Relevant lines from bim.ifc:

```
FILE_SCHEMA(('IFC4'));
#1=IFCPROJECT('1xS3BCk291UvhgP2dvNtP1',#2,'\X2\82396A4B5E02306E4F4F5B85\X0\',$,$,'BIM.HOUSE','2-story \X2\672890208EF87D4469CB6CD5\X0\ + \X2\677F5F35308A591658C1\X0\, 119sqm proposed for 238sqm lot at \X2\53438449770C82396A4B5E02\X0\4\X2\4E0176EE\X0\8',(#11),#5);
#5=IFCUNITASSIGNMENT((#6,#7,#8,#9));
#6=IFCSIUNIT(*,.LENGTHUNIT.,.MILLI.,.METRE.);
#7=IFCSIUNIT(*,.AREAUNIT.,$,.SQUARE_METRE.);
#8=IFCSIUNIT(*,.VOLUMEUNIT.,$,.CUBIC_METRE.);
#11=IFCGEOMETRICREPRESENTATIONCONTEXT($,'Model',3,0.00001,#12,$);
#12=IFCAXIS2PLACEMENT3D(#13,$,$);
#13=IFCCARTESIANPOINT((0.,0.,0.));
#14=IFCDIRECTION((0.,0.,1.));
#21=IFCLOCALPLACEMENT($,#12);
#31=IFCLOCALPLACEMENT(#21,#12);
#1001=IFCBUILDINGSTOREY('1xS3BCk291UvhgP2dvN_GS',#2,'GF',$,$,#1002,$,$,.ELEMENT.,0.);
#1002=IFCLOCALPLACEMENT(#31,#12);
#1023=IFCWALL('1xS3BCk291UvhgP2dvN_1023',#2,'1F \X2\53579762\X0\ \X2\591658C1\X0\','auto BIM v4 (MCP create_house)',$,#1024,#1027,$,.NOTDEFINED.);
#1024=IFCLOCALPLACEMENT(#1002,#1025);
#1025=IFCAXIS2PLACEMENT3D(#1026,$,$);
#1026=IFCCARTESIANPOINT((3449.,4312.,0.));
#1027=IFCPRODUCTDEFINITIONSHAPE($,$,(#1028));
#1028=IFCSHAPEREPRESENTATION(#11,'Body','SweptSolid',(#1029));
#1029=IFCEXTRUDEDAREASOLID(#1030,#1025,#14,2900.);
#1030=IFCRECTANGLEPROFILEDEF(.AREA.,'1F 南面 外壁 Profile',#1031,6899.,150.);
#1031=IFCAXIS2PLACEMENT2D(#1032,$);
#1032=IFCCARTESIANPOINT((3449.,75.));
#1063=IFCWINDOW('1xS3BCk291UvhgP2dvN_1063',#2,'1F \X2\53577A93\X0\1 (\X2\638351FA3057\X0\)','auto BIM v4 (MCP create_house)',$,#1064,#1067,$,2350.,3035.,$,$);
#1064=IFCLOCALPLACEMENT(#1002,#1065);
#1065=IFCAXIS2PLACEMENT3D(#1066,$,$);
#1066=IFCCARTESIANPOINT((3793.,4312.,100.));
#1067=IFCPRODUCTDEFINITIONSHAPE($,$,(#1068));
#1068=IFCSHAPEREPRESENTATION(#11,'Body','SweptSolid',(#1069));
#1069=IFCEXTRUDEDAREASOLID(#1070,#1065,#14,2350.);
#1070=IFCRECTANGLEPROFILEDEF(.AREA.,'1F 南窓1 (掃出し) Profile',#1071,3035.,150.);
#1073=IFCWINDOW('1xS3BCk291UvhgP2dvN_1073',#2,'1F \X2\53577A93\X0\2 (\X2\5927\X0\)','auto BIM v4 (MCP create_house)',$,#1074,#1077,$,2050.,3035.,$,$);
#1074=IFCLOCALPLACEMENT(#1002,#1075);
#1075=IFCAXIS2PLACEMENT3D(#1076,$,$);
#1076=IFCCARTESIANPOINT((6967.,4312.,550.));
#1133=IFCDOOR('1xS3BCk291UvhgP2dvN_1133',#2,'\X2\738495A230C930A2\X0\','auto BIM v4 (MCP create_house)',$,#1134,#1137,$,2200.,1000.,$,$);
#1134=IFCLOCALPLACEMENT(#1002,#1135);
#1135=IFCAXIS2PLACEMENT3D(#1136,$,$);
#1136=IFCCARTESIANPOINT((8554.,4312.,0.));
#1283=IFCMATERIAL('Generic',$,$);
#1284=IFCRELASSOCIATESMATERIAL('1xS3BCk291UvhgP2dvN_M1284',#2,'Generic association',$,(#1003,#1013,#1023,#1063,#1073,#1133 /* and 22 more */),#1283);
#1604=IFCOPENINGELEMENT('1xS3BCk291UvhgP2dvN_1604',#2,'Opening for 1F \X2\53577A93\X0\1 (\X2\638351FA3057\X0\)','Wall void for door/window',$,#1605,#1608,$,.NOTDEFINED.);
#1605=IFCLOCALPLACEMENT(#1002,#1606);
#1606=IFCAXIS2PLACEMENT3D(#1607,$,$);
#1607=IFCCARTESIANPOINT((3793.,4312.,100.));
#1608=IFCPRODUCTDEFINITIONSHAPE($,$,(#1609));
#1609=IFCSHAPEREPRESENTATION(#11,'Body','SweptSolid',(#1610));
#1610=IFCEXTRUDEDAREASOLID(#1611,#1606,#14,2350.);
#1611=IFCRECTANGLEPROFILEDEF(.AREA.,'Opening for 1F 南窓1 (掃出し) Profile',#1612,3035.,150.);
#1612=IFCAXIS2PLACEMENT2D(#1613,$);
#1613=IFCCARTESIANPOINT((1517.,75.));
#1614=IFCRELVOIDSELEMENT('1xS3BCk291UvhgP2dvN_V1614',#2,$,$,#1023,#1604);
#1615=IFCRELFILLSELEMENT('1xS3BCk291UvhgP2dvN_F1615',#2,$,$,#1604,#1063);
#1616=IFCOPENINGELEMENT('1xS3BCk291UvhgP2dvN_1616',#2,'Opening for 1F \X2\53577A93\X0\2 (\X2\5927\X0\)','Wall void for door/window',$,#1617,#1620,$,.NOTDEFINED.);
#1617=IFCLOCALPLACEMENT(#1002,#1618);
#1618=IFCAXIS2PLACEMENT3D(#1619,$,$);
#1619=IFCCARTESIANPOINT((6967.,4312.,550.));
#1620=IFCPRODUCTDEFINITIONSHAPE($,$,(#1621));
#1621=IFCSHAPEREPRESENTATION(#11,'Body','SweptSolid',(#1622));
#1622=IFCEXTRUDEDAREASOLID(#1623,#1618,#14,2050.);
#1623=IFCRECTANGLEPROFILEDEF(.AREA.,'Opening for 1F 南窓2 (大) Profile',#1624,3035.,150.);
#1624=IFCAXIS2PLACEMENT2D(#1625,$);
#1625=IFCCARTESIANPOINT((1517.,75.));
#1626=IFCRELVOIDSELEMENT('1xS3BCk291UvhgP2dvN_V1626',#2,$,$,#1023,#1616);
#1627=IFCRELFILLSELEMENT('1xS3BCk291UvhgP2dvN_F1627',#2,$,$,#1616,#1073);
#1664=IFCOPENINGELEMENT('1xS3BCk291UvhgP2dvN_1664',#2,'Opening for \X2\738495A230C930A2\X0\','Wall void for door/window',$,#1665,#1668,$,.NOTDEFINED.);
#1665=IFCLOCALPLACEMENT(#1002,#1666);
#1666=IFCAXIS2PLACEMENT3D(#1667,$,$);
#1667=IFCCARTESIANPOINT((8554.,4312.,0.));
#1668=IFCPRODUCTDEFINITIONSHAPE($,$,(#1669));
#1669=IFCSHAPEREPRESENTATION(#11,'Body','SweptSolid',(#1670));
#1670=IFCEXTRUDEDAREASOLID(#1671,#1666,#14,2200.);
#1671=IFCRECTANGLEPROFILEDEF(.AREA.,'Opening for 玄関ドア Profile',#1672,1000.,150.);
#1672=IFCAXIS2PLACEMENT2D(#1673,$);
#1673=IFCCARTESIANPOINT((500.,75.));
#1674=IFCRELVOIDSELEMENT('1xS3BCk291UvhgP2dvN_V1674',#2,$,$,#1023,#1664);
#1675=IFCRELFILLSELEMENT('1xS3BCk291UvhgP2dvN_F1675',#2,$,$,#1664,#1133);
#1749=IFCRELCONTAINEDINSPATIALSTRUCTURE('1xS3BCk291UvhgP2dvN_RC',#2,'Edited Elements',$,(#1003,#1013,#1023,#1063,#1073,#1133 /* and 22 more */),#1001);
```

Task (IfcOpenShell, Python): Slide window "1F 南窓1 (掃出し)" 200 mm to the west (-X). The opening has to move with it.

```python
import ifcopenshell
import ifcopenshell.api.geometry
import ifcopenshell.util.placement
import ifcopenshell.util.unit

model = ifcopenshell.open("bim.ifc")
unit_scale = ifcopenshell.util.unit.calculate_unit_scale(model)

window = model.by_guid("1xS3BCk291UvhgP2dvN_1063")
opening = window.FillsVoids[0].RelatingOpeningElement
wall = opening.VoidsElements[0].RelatingBuildingElement

wall_matrix = ifcopenshell.util.placement.get_local_placement(wall.ObjectPlacement)
shift = wall_matrix[:3, 0] * -0.2 / unit_scale
before = ifcopenshell.util.placement.get_local_placement(window.ObjectPlacement)[:3, 3].copy()

# The window is not placed relative to its opening, so move both.
for product in (opening, window):
    matrix = ifcopenshell.util.placement.get_local_placement(product.ObjectPlacement)
    matrix[:3, 3] += shift
    ifcopenshell.api.geometry.edit_object_placement(model, product=product, matrix=matrix, is_si=False)

after = ifcopenshell.util.placement.get_local_placement(window.ObjectPlacement)[:3, 3]
print("window moved by", (after - before).round(3) + 0.0)

model.write("bim_updated.ifc")
```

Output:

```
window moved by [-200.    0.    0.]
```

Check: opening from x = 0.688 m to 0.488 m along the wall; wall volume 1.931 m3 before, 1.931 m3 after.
